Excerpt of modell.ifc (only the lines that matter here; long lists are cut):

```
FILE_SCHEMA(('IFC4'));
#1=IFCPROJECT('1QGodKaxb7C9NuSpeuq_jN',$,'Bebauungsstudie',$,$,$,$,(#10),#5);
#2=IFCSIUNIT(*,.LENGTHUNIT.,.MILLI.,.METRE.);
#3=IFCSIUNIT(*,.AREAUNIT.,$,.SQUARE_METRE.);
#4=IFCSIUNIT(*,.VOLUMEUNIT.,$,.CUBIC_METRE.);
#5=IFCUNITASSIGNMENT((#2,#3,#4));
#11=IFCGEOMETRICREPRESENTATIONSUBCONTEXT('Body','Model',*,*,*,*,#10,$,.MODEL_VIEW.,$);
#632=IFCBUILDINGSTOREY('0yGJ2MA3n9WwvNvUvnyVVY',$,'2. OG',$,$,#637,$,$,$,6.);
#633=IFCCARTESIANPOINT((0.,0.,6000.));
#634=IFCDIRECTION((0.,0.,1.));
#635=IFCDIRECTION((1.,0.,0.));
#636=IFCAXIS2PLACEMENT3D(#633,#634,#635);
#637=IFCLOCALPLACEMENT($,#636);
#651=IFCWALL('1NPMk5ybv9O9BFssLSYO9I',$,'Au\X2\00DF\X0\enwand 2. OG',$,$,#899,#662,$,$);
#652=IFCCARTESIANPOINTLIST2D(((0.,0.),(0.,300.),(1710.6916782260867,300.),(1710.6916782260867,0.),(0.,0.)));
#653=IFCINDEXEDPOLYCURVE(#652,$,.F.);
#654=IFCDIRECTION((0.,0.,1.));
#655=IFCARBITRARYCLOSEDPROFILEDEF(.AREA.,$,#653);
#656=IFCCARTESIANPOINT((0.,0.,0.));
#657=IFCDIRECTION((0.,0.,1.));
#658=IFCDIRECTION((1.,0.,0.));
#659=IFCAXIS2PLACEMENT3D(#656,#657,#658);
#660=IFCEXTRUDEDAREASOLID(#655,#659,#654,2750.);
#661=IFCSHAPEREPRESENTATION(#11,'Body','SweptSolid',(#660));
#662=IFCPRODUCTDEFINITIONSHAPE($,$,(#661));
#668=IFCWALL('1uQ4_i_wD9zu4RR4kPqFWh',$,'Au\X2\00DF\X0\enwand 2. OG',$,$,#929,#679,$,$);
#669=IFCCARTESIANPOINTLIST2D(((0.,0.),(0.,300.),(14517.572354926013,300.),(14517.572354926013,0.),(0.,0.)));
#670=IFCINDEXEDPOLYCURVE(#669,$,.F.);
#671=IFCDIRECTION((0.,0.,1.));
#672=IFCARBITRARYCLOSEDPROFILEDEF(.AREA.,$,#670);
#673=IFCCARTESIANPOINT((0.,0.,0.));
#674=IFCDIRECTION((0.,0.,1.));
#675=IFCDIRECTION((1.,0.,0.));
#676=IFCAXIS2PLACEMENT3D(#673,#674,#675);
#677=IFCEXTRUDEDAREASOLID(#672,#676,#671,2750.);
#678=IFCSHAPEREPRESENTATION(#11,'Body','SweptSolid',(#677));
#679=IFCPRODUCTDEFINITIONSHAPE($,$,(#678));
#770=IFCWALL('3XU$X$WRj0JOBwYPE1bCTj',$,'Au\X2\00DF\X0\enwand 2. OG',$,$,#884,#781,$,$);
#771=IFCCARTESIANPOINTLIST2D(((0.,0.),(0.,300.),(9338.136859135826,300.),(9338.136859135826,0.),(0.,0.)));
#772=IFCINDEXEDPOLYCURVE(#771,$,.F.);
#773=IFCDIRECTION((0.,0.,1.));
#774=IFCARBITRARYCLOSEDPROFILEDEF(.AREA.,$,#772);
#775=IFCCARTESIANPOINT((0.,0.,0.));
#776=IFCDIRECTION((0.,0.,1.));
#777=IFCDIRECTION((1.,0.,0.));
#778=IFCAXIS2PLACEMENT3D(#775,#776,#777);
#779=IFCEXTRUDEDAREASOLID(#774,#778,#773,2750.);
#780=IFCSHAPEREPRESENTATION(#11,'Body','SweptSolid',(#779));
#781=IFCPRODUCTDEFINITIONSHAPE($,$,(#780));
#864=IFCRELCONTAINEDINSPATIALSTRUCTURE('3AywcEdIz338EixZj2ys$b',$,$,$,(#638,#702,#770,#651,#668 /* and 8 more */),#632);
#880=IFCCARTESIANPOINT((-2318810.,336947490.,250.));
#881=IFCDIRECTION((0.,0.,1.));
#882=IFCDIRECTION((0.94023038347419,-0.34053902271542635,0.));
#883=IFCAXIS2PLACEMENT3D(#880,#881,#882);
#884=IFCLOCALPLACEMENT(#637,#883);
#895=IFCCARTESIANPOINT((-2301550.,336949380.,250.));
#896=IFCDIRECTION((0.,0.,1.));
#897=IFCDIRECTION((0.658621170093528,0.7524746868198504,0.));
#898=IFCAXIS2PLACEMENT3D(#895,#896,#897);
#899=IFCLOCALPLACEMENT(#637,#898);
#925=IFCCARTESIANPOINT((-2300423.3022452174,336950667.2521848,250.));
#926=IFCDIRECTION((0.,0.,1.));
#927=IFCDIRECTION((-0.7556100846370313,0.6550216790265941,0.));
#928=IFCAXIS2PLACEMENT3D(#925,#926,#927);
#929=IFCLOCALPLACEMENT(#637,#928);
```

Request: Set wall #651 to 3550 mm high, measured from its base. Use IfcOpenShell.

```python
import ifcopenshell
import ifcopenshell.geom
import ifcopenshell.util.representation
import ifcopenshell.util.shape
import ifcopenshell.util.unit

model = ifcopenshell.open("modell.ifc")
unit_scale = ifcopenshell.util.unit.calculate_unit_scale(model)
settings = ifcopenshell.geom.settings()


def volume(element):
    """Net volume in cubic metres, openings subtracted."""
    shape = ifcopenshell.geom.create_shape(settings, element)
    return ifcopenshell.util.shape.get_volume(shape.geometry)


wall = model.by_id(651)
before = volume(wall)

body = ifcopenshell.util.representation.get_representation(wall, "Model", "Body")
solid = body.Items[0]
old_height = solid.Depth
solid.Depth = 3.55 / unit_scale
after = volume(wall)

print(f"height {old_height:g} -> {solid.Depth:g}, volume {before:.3f} -> {after:.3f} m3")

model.write("modell-out.ifc")
```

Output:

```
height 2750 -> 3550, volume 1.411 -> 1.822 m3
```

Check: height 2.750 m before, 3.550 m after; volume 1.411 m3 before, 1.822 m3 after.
